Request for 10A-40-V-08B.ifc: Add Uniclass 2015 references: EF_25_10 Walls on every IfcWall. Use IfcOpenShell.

First a look at what the model holds.

```python
import ifcopenshell

model = ifcopenshell.open("10A-40-V-08B.ifc")
print(model.schema)
print("classifications:", [c.Name for c in model.by_type("IfcClassification")])
for ifc_class in ("IfcDoor", "IfcRoof", "IfcStair", "IfcWall", "IfcWindow"):
    print(ifc_class, len(model.by_type(ifc_class)))
```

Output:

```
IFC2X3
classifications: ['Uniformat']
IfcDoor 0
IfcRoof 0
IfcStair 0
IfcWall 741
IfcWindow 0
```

```python
import ifcopenshell
import ifcopenshell.api.classification

model = ifcopenshell.open("10A-40-V-08B.ifc")

# IFC2X3 requires Source and Edition and has no link from the project to the system.
system = model.create_entity("IfcClassification", Source="NBS", Edition="2015", Name="Uniclass 2015")

codes = {
    "IfcWall": ("EF_25_10", "Walls"),
}
for ifc_class, (code, name) in codes.items():
    products = model.by_type(ifc_class)
    ifcopenshell.api.classification.add_reference(
        model, products=products, classification=system, identification=code, name=name
    )
    print(code, len(products))

model.write("10A-40-V-08B_edited.ifc")
```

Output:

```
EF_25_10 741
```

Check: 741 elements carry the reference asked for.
